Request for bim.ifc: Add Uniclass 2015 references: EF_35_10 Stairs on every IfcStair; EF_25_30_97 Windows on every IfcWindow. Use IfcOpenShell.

First a look at what the model holds.

```python
import ifcopenshell

model = ifcopenshell.open("bim.ifc")
print(model.schema)
print("classifications:", [c.Name for c in model.by_type("IfcClassification")])
for ifc_class in ("IfcDoor", "IfcRoof", "IfcStair", "IfcWall", "IfcWindow"):
    print(ifc_class, len(model.by_type(ifc_class)))
```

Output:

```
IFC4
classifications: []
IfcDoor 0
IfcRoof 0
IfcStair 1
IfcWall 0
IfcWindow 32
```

```python
import ifcopenshell
import ifcopenshell.api.classification

model = ifcopenshell.open("bim.ifc")

system = ifcopenshell.api.classification.add_classification(model, classification="Uniclass 2015")

codes = {
    "IfcStair": ("EF_35_10", "Stairs"),
    "IfcWindow": ("EF_25_30_97", "Windows"),
}
for ifc_class, (code, name) in codes.items():
    products = model.by_type(ifc_class)
    ifcopenshell.api.classification.add_reference(
        model, products=products, classification=system, identification=code, name=name
    )
    print(code, len(products))

model.write("bim_rev.ifc")
```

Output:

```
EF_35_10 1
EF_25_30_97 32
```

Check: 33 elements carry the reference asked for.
